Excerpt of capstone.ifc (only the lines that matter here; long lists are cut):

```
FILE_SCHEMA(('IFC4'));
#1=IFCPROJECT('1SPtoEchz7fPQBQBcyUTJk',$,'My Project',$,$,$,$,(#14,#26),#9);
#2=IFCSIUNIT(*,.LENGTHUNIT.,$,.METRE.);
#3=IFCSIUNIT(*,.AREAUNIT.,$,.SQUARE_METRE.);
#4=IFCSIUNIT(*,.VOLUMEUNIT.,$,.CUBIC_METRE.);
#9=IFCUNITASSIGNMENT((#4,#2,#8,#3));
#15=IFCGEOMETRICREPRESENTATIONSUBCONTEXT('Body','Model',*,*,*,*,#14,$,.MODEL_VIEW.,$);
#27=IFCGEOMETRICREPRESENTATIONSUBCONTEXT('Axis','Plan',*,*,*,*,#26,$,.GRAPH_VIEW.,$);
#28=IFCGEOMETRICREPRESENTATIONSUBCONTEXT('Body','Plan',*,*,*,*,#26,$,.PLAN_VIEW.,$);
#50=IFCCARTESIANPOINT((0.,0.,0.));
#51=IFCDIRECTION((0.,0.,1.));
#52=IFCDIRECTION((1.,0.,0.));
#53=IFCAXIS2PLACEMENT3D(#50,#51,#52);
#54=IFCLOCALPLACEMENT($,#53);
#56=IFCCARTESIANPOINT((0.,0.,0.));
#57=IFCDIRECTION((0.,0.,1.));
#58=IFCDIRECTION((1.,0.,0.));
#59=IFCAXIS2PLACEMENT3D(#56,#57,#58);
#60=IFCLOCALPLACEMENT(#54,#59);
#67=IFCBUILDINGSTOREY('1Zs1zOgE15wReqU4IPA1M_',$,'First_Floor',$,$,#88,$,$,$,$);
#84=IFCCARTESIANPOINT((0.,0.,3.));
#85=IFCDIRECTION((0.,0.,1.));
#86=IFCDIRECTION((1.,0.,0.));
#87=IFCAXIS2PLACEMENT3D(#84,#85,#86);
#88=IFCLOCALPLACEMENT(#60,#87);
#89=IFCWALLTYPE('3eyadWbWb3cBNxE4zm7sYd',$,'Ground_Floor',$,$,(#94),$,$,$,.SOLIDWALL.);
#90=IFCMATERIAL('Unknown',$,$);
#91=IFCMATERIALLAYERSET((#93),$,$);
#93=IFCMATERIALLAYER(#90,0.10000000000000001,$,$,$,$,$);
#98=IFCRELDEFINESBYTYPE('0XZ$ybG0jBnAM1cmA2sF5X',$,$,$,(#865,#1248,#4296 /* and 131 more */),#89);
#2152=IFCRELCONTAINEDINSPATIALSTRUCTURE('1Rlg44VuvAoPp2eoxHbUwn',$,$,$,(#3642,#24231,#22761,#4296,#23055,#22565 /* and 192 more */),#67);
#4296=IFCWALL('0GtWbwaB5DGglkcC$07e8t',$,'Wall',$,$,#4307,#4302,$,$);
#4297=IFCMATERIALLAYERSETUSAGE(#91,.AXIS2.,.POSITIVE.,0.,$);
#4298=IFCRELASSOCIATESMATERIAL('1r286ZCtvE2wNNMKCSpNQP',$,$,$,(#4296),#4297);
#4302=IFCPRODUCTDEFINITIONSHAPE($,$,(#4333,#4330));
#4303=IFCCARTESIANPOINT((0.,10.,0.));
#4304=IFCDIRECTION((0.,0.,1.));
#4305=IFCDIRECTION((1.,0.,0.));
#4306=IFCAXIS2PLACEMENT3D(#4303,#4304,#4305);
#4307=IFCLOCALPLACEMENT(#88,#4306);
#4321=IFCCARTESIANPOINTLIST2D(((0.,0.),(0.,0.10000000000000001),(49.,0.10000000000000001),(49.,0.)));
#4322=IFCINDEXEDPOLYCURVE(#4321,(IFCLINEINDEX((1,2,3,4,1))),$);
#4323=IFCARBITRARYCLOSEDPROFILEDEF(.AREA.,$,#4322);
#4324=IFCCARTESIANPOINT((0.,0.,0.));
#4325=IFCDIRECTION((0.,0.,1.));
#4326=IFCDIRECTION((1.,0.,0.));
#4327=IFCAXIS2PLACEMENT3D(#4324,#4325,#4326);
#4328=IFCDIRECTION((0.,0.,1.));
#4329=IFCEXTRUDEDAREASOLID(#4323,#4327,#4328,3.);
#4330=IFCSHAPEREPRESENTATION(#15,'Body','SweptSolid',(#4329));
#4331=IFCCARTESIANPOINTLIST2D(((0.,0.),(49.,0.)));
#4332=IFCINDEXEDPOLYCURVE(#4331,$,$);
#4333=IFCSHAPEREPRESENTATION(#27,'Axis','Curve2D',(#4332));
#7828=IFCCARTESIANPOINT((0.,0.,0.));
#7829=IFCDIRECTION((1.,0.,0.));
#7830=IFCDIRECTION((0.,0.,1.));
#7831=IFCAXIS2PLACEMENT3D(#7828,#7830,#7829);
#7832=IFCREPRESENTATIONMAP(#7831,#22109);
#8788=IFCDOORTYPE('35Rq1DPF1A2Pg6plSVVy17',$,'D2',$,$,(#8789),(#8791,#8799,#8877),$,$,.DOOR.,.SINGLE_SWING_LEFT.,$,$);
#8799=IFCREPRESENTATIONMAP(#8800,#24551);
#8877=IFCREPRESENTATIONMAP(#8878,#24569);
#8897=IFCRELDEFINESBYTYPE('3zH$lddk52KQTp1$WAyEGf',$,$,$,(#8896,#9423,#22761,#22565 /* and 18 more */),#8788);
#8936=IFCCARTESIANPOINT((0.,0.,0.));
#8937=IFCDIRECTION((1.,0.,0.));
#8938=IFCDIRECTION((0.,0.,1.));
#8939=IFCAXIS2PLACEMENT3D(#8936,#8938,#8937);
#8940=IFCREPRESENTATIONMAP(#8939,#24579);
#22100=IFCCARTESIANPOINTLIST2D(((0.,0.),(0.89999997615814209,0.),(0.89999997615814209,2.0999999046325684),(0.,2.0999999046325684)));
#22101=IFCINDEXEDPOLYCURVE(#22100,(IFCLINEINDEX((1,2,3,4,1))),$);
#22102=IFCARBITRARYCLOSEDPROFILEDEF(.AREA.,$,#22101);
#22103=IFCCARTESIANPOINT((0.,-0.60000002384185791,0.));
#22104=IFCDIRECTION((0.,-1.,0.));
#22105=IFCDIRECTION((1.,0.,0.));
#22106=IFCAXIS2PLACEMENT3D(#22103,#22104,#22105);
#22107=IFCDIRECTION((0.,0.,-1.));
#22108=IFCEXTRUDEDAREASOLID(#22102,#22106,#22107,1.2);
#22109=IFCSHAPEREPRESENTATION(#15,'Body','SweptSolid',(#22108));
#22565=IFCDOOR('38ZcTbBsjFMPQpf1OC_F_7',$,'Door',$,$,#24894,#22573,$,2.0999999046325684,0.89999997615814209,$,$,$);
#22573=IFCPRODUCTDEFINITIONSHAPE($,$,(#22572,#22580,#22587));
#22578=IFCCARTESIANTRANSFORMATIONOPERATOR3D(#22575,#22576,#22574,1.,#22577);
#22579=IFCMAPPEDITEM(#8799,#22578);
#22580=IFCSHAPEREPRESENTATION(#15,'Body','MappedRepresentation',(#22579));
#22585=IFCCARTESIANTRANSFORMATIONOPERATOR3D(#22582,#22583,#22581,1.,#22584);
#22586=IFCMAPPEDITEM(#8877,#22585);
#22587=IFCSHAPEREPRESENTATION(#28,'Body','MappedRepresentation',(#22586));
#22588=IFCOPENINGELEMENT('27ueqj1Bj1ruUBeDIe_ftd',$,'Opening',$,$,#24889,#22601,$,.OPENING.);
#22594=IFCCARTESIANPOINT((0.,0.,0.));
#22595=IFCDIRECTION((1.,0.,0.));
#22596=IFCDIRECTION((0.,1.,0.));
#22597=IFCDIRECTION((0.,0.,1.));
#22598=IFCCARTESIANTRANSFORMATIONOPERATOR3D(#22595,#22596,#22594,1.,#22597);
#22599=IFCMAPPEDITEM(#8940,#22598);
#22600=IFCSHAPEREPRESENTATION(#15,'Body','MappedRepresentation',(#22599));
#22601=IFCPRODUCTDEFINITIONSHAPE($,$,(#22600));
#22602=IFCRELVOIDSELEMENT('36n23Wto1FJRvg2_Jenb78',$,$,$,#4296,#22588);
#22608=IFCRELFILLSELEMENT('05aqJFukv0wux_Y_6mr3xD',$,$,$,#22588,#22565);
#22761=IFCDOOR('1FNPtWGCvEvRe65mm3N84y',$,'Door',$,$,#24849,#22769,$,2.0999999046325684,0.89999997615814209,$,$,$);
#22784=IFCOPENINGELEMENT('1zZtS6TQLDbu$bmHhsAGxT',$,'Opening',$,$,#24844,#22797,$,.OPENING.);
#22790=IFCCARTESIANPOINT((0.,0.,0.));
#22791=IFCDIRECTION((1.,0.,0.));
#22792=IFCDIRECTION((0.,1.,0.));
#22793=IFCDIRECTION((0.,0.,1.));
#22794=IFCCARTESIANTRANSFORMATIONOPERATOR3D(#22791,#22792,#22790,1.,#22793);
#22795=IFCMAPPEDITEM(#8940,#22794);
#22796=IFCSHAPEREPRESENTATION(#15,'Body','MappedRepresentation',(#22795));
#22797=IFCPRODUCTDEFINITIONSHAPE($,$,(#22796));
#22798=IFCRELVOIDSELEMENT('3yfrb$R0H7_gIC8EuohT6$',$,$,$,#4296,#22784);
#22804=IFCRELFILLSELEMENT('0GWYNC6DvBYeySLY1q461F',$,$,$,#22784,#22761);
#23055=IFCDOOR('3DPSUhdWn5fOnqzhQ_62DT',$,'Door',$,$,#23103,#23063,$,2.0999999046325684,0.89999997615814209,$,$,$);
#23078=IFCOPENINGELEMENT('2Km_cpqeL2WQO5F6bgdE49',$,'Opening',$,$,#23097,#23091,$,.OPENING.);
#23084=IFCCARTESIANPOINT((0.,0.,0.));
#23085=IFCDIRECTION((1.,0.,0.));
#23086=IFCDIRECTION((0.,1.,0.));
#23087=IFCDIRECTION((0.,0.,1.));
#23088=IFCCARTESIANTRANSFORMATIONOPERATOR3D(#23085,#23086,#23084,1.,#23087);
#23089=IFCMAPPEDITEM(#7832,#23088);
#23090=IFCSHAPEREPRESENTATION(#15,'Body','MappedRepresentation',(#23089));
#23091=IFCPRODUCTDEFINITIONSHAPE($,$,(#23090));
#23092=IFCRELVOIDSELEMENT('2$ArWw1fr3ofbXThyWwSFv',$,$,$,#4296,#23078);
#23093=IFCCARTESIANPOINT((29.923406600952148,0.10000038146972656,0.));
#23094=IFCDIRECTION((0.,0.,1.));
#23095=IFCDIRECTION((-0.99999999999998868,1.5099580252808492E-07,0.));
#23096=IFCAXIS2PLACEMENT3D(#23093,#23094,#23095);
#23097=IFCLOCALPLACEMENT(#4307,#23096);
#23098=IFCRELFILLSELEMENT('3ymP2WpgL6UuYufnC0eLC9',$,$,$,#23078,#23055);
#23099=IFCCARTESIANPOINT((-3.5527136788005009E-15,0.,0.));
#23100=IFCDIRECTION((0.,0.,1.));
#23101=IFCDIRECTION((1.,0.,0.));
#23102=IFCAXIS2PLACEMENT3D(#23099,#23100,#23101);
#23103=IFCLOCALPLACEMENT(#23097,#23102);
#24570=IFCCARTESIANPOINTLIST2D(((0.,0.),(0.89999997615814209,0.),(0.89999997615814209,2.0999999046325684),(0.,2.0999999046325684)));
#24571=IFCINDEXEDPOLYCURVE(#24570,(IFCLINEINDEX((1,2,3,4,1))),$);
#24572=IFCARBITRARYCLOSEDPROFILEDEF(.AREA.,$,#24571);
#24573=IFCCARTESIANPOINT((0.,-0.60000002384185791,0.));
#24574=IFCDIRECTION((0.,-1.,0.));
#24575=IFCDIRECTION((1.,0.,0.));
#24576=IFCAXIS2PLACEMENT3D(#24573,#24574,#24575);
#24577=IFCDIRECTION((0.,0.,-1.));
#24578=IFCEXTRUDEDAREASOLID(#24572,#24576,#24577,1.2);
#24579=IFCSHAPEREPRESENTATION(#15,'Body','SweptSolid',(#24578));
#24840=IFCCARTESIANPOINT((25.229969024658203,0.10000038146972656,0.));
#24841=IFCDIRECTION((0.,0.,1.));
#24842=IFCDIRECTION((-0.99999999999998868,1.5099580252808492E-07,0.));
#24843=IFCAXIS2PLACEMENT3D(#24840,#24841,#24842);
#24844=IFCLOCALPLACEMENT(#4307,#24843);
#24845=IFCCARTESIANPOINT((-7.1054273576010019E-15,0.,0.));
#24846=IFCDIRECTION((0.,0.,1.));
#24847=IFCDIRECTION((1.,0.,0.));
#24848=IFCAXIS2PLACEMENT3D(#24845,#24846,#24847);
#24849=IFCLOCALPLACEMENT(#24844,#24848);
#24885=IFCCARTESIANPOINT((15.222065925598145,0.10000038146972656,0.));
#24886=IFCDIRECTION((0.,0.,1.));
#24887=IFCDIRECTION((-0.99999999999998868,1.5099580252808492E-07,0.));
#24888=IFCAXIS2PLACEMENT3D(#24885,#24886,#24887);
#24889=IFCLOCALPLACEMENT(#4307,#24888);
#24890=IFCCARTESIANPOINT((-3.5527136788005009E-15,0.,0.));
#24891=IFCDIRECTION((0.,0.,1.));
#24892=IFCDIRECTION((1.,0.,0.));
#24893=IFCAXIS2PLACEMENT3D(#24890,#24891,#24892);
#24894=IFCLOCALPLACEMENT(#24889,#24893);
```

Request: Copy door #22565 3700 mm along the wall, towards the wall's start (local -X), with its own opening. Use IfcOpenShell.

```python
import ifcopenshell
import ifcopenshell.api.feature
import ifcopenshell.api.geometry
import ifcopenshell.api.root
import ifcopenshell.geom
import ifcopenshell.util.element
import ifcopenshell.util.placement
import ifcopenshell.util.shape

model = ifcopenshell.open("capstone.ifc")
settings = ifcopenshell.geom.settings()


def volume(element):
    """Net volume in cubic metres, openings subtracted."""
    shape = ifcopenshell.geom.create_shape(settings, element)
    return ifcopenshell.util.shape.get_volume(shape.geometry)


door = model.by_guid("38ZcTbBsjFMPQpf1OC_F_7")
opening = door.FillsVoids[0].RelatingOpeningElement
wall = opening.VoidsElements[0].RelatingBuildingElement
before = volume(wall)
shift = ifcopenshell.util.placement.get_local_placement(wall.ObjectPlacement)[:3, 0] * -3.7

# copy_class copies the void relationship, type, container and properties, but no geometry.
new_opening = ifcopenshell.api.root.copy_class(model, product=opening)
new_opening.Representation = ifcopenshell.util.element.copy_deep(
    model, opening.Representation, exclude=["IfcGeometricRepresentationContext", "IfcRepresentationMap"]
)
new_door = ifcopenshell.api.root.copy_class(model, product=door)
new_door.Representation = ifcopenshell.util.element.copy_deep(
    model, door.Representation, exclude=["IfcGeometricRepresentationContext", "IfcRepresentationMap"]
)
ifcopenshell.api.feature.add_filling(model, opening=new_opening, element=new_door)

for old, new in ((opening, new_opening), (door, new_door)):
    matrix = ifcopenshell.util.placement.get_local_placement(old.ObjectPlacement)
    matrix[:3, 3] += shift
    ifcopenshell.api.geometry.edit_object_placement(model, product=new, matrix=matrix, is_si=False)

after = volume(wall)

print(f"wall volume {before:.3f} -> {after:.3f} m3")

model.write("capstone-out.ifc")
```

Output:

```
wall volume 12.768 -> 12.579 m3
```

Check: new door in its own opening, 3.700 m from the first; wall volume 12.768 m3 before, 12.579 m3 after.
